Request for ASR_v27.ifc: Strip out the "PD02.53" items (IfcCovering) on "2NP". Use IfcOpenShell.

First a look at what the model holds.

```python
import ifcopenshell
import ifcopenshell.util.element

model = ifcopenshell.open("ASR_v27.ifc")
print(model.schema)
storey = next(s for s in model.by_type("IfcBuildingStorey") if s.Name == "2NP")
coverings = [e for e in ifcopenshell.util.element.get_decomposition(storey) if e.is_a("IfcCovering")]
seen = {}
for e in coverings:
    element_type = ifcopenshell.util.element.get_type(e)
    name = element_type.Name if element_type not in (None, e) else None
    seen[name] = seen.get(name, 0) + 1
for name, count in sorted(seen.items(), key=str):
    print(count, "x", name)
```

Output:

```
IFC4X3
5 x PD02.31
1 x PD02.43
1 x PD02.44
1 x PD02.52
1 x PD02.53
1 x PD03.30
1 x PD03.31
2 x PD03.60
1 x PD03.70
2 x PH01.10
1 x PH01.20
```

```python
import ifcopenshell
import ifcopenshell.api.root
import ifcopenshell.util.element

model = ifcopenshell.open("ASR_v27.ifc")

storey = next(s for s in model.by_type("IfcBuildingStorey") if s.Name == "2NP")
coverings = [e for e in ifcopenshell.util.element.get_decomposition(storey) if e.is_a("IfcCovering")]
targets = [e for e in coverings if (t := ifcopenshell.util.element.get_type(e)) not in (None, e) and t.Name == "PD02.53"]

for e in targets:
    ifcopenshell.api.root.remove_product(model, product=e)
print(len(targets), "removed")

model.write("ASR_v27_edited.ifc")
```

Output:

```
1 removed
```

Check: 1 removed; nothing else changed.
